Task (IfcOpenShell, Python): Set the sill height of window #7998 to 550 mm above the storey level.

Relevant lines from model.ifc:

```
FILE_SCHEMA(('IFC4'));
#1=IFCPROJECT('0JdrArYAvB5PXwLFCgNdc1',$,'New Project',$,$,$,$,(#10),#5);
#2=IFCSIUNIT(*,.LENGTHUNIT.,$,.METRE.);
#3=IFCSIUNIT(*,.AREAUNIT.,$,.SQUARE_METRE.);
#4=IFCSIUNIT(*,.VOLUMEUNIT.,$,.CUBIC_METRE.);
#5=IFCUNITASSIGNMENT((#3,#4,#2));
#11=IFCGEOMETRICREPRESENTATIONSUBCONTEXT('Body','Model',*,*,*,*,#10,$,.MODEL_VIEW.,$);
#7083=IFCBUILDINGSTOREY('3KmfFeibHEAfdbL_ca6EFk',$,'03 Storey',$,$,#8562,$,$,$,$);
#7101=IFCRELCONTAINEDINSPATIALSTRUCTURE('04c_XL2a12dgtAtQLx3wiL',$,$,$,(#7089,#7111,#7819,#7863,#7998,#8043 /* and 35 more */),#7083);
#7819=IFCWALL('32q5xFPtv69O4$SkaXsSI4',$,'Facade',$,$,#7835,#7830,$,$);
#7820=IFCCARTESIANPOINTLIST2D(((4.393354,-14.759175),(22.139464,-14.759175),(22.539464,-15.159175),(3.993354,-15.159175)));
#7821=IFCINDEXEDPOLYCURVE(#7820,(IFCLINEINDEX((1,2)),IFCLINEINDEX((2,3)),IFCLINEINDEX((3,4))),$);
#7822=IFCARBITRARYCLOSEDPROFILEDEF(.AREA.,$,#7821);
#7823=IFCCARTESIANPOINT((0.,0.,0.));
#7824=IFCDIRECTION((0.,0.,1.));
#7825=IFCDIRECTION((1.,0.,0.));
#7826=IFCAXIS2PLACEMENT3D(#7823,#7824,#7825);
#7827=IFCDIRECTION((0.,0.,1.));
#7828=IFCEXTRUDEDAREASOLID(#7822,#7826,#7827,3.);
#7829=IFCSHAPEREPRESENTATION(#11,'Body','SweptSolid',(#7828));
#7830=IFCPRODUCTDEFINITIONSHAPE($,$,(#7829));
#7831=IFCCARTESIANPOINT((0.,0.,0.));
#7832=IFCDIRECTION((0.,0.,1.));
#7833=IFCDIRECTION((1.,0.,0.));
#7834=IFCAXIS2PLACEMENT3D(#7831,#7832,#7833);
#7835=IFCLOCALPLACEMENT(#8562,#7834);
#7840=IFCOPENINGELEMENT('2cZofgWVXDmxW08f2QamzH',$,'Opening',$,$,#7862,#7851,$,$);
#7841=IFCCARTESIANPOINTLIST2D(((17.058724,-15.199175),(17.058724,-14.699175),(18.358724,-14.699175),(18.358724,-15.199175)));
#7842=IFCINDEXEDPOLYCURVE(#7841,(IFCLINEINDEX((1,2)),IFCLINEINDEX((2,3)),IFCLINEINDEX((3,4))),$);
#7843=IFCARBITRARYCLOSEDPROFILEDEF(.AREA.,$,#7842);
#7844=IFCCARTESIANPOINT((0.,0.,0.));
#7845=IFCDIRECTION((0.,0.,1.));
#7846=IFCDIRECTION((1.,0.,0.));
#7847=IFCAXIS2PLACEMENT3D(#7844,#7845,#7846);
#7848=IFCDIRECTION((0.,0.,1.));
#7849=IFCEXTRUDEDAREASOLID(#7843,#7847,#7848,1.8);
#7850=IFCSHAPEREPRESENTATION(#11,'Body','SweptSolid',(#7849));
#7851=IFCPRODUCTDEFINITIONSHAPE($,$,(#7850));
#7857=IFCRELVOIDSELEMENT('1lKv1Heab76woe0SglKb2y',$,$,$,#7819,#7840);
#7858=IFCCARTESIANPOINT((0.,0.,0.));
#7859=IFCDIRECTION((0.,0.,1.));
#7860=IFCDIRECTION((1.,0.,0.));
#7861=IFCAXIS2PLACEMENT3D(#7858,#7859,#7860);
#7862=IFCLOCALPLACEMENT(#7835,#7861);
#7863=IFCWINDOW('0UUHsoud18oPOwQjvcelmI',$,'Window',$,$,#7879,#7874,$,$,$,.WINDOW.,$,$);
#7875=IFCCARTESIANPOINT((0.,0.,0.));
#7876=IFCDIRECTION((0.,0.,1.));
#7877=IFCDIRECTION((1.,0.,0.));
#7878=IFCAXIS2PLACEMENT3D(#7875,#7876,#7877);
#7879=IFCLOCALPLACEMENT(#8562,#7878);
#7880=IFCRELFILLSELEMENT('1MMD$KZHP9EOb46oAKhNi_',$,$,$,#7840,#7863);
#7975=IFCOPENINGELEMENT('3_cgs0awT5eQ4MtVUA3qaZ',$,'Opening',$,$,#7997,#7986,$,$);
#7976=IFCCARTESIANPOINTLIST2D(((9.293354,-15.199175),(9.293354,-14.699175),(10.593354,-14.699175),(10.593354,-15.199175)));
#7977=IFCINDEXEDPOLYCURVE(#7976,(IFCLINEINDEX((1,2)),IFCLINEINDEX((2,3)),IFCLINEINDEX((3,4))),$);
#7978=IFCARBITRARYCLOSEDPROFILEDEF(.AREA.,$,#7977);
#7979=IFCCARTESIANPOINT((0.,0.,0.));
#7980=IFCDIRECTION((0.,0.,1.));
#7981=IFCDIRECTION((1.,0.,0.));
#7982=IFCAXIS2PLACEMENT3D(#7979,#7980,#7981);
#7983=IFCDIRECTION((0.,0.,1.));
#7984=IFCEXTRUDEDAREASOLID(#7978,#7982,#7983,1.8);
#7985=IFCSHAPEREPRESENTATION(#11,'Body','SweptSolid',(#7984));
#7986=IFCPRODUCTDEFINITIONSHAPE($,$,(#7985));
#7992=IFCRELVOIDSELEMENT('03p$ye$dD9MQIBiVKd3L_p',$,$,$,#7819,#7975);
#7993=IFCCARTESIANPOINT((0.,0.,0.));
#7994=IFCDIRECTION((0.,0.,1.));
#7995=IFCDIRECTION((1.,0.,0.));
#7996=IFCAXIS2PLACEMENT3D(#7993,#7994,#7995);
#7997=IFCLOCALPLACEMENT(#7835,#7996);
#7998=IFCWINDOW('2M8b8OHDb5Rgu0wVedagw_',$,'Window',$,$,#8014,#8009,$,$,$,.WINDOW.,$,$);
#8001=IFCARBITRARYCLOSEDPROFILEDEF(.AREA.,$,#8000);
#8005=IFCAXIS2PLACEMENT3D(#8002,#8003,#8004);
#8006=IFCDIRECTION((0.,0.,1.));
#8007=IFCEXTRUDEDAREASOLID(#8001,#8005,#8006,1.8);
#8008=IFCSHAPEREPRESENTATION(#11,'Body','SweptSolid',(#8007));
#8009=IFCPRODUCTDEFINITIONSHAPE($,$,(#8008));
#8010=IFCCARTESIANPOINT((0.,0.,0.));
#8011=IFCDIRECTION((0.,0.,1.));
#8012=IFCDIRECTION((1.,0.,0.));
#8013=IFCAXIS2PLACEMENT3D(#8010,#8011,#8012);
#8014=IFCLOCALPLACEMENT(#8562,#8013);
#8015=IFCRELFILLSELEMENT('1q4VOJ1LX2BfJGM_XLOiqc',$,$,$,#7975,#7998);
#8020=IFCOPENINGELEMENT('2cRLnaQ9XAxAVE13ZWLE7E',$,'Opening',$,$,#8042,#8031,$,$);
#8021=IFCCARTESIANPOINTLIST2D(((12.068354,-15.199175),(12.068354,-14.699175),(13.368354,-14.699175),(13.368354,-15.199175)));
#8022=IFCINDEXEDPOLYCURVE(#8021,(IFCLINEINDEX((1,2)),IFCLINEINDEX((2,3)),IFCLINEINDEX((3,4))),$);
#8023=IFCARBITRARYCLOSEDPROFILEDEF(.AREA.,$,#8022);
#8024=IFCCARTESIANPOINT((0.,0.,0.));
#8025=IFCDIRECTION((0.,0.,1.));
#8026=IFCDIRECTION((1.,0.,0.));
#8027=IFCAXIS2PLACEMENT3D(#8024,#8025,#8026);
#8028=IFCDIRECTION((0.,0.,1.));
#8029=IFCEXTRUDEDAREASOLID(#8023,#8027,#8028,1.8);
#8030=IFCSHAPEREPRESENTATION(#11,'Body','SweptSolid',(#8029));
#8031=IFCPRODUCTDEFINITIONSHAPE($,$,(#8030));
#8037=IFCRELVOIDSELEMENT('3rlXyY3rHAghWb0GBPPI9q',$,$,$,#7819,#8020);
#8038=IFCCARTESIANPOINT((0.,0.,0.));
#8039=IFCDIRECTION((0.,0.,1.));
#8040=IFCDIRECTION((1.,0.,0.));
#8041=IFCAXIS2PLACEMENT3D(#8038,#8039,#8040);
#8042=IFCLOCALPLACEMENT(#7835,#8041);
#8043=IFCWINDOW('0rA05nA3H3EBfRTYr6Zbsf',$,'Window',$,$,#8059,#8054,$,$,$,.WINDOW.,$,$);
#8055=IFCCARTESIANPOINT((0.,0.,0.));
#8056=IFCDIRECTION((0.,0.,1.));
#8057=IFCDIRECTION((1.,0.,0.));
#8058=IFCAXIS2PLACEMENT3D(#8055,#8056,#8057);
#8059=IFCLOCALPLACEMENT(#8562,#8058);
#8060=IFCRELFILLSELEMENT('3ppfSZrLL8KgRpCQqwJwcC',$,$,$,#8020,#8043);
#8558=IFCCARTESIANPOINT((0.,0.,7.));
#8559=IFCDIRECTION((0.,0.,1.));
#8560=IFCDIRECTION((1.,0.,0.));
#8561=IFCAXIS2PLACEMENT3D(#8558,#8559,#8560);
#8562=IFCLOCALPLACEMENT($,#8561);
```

```python
import numpy as np
import ifcopenshell
import ifcopenshell.api.geometry
import ifcopenshell.geom
import ifcopenshell.util.element
import ifcopenshell.util.placement
import ifcopenshell.util.shape
import ifcopenshell.util.unit

model = ifcopenshell.open("model.ifc")
unit_scale = ifcopenshell.util.unit.calculate_unit_scale(model)

window = model.by_id(7998)
opening = window.FillsVoids[0].RelatingOpeningElement
storey = ifcopenshell.util.element.get_container(window, ifc_class="IfcBuildingStorey")
level = ifcopenshell.util.placement.get_local_placement(storey.ObjectPlacement)[2, 3]

# The opening's origin need not be at the sill, so measure its lowest point.
shape = ifcopenshell.geom.create_shape(ifcopenshell.geom.settings(), opening)
bottom = ifcopenshell.util.shape.get_shape_bottom_elevation(shape, shape.geometry) / unit_scale
dz = level + 0.55 - bottom

shift = np.array([0.0, 0.0, dz])
# The window is not placed relative to its opening, so move both.
for product in (opening, window):
    matrix = ifcopenshell.util.placement.get_local_placement(product.ObjectPlacement)
    matrix[:3, 3] += shift
    ifcopenshell.api.geometry.edit_object_placement(model, product=product, matrix=matrix, is_si=False)

print(f"moved by {dz * unit_scale:+.3f} m")

model.write("model_updated.ifc")
```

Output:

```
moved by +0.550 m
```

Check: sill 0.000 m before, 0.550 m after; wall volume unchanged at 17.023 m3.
